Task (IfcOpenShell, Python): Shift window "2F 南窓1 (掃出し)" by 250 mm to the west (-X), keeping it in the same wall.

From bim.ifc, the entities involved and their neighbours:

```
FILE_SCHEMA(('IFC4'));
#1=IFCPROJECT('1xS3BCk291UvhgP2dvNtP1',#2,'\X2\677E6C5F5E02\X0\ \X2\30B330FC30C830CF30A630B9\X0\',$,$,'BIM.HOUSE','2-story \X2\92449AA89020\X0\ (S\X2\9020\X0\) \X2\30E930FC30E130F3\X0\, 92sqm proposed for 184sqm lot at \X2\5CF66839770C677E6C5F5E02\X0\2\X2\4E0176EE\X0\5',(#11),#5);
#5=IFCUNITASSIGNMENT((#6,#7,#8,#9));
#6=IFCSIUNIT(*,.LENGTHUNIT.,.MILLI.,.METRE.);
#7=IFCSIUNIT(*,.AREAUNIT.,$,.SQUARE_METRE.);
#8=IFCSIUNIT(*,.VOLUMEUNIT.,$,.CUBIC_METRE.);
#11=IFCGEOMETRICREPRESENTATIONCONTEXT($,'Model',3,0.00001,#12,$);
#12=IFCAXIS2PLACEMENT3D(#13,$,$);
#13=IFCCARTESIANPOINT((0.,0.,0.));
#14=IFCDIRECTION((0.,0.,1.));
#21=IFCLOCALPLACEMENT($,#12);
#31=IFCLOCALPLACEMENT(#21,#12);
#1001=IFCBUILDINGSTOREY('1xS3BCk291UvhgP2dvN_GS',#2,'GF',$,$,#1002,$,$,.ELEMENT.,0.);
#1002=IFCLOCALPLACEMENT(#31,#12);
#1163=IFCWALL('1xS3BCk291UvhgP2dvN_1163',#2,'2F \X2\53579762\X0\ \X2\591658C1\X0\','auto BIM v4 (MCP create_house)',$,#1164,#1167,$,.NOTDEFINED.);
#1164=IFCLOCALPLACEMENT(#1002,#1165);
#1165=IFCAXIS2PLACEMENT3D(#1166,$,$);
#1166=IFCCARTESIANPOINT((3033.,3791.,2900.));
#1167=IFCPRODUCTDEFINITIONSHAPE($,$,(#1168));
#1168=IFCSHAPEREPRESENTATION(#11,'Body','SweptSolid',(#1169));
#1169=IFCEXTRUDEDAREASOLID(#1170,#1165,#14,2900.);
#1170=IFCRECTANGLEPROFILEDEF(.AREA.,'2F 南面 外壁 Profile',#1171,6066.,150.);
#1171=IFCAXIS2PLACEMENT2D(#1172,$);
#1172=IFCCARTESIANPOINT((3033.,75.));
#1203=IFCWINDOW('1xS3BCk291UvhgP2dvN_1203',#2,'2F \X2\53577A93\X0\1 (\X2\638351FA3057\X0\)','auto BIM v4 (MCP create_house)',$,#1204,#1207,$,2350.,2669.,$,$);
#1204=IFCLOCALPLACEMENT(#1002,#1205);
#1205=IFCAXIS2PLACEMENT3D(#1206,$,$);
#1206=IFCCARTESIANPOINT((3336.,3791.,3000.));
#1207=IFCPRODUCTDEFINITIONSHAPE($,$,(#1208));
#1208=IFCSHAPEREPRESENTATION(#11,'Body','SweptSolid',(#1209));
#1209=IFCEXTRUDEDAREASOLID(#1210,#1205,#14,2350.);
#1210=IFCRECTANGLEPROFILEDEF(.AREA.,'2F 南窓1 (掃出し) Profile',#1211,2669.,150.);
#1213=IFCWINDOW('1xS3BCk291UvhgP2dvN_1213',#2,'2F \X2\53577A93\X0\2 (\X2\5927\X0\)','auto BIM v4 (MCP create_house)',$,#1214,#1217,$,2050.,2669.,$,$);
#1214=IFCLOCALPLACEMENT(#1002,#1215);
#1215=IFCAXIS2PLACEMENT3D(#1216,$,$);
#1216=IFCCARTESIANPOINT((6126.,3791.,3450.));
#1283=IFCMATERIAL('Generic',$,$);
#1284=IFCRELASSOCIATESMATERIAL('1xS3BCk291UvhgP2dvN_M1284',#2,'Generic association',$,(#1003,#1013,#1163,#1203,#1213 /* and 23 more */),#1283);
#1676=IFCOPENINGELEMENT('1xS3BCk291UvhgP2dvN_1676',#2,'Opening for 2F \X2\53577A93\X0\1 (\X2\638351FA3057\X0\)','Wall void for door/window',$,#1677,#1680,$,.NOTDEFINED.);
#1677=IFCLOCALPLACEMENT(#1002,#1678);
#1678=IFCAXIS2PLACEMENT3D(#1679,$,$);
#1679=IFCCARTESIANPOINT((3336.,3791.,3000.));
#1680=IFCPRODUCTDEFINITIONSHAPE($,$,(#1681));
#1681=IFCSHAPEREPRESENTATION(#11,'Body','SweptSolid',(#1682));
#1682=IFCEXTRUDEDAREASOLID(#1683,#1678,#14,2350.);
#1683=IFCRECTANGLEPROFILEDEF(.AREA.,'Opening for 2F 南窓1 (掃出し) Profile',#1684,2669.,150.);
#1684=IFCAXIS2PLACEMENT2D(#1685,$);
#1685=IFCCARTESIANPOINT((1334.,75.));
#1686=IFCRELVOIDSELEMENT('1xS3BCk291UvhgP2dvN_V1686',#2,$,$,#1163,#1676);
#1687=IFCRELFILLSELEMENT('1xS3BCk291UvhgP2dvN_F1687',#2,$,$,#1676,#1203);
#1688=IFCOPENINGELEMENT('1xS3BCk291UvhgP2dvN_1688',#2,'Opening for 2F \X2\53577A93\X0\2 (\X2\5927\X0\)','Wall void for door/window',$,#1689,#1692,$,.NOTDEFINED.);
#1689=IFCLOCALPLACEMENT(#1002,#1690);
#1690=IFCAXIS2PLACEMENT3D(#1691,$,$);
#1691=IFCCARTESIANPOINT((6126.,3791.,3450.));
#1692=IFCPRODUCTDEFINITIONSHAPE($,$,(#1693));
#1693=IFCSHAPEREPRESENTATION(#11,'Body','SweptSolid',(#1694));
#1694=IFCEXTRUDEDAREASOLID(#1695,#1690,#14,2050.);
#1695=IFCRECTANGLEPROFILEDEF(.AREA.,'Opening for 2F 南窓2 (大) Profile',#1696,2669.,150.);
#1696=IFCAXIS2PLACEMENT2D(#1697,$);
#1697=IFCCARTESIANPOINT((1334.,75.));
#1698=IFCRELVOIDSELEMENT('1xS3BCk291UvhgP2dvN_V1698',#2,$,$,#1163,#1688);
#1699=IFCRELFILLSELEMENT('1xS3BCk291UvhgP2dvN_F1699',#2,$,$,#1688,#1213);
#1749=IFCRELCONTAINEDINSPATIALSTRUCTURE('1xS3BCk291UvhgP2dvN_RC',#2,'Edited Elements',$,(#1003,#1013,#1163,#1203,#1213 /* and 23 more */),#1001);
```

```python
import ifcopenshell
import ifcopenshell.api.geometry
import ifcopenshell.util.placement

model = ifcopenshell.open("bim.ifc")

window = model.by_guid("1xS3BCk291UvhgP2dvN_1203")
opening = window.FillsVoids[0].RelatingOpeningElement
wall = opening.VoidsElements[0].RelatingBuildingElement

wall_matrix = ifcopenshell.util.placement.get_local_placement(wall.ObjectPlacement)
shift = wall_matrix[:3, 0] * -250.0
before = ifcopenshell.util.placement.get_local_placement(window.ObjectPlacement)[:3, 3].copy()

# The window is not placed relative to its opening, so move both.
for product in (opening, window):
    matrix = ifcopenshell.util.placement.get_local_placement(product.ObjectPlacement)
    matrix[:3, 3] += shift
    ifcopenshell.api.geometry.edit_object_placement(model, product=product, matrix=matrix, is_si=False)

after = ifcopenshell.util.placement.get_local_placement(window.ObjectPlacement)[:3, 3]
print("window moved by", (after - before).round(3) + 0.0)

model.write("bim_edited.ifc")
```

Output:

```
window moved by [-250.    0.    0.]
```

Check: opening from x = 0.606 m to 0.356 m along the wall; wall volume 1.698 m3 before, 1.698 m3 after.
